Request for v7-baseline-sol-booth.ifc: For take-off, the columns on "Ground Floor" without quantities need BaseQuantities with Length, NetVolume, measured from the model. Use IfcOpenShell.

First a look at what the model holds.

```python
import ifcopenshell
import ifcopenshell.util.element
import ifcopenshell.util.unit

model = ifcopenshell.open("v7-baseline-sol-booth.ifc")
print(model.schema)
for unit_type in ("LENGTHUNIT", "AREAUNIT", "VOLUMEUNIT"):
    print(unit_type, ifcopenshell.util.unit.calculate_unit_scale(model, unit_type))
storey = next(s for s in model.by_type("IfcBuildingStorey") if s.Name == "Ground Floor")
columns = [e for e in ifcopenshell.util.element.get_decomposition(storey) if e.is_a("IfcColumn")]
for e in sorted(columns, key=lambda e: e.id()):
    print(e.id(), e.is_a(), e.Name, list(ifcopenshell.util.element.get_psets(e, qtos_only=True)), sep=" | ")
```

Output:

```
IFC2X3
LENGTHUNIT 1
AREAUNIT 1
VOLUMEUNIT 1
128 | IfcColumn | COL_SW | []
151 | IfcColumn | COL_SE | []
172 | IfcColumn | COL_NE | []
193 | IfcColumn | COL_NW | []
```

```python
import ifcopenshell
import ifcopenshell.api.pset
import ifcopenshell.geom
import ifcopenshell.util.element
import ifcopenshell.util.shape
import ifcopenshell.util.unit

model = ifcopenshell.open("v7-baseline-sol-booth.ifc")
unit_scale = ifcopenshell.util.unit.calculate_unit_scale(model)
volume_scale = ifcopenshell.util.unit.calculate_unit_scale(model, "VOLUMEUNIT")
settings = ifcopenshell.geom.settings()

storey = next(s for s in model.by_type("IfcBuildingStorey") if s.Name == "Ground Floor")
columns = [e for e in ifcopenshell.util.element.get_decomposition(storey) if e.is_a("IfcColumn")]

for e in sorted(columns, key=lambda e: e.id()):
    if ifcopenshell.util.element.get_psets(e, qtos_only=True, should_inherit=False):
        continue
    # Geometry comes back in metres, in the element's own axes.
    shape = ifcopenshell.geom.create_shape(settings, e)
    values = {
        "Length": ifcopenshell.util.shape.get_z(shape.geometry) / unit_scale,
        "NetVolume": ifcopenshell.util.shape.get_volume(shape.geometry) / volume_scale,
    }
    qto = ifcopenshell.api.pset.add_qto(model, product=e, name="BaseQuantities")
    ifcopenshell.api.pset.edit_qto(model, qto=qto, properties=values)
    print(e.id(), {k: round(v, 3) for k, v in values.items()})

model.write("v7-baseline-sol-booth_edited.ifc")
```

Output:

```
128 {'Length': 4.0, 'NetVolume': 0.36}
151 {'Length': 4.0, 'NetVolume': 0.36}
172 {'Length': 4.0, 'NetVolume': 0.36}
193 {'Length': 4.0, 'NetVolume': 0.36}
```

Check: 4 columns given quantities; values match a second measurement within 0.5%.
